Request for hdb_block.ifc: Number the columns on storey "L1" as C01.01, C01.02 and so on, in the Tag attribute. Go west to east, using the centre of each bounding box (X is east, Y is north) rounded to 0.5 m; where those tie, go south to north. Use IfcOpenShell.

First a look at what the model holds.

```python
import ifcopenshell
import ifcopenshell.util.element
import ifcopenshell.util.placement

model = ifcopenshell.open("hdb_block.ifc")
print(model.schema)
storey = next(s for s in model.by_type("IfcBuildingStorey") if s.Name == "L1")
columns = [e for e in ifcopenshell.util.element.get_decomposition(storey) if e.is_a("IfcColumn")]
for e in sorted(columns, key=lambda e: e.id()):
    origin = ifcopenshell.util.placement.get_local_placement(e.ObjectPlacement)[:3, 3]
    print(e.id(), e.Tag, e.Name, origin.round(2) + 0.0, sep=" | ")
```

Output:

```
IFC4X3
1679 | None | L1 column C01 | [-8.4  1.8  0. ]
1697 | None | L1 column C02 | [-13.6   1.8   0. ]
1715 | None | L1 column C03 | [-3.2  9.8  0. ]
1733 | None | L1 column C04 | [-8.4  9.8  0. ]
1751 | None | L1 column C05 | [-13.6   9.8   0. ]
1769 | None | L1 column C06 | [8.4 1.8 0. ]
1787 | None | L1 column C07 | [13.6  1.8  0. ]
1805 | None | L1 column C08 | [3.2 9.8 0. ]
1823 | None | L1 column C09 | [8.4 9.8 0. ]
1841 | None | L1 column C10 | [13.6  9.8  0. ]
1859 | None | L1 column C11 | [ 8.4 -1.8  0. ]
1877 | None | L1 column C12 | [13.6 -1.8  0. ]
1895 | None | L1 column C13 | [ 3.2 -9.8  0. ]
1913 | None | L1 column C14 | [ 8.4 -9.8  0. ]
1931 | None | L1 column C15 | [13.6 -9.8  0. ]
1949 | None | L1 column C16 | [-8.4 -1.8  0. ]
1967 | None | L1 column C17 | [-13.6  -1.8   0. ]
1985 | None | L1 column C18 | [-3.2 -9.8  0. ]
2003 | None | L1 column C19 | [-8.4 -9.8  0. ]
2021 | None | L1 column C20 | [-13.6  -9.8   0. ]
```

```python
import ifcopenshell
import ifcopenshell.geom
import ifcopenshell.util.element
import ifcopenshell.util.shape

model = ifcopenshell.open("hdb_block.ifc")
settings = ifcopenshell.geom.settings()
settings.set("use-world-coords", True)


def centre(element):
    shape = ifcopenshell.geom.create_shape(settings, element)
    return ifcopenshell.util.shape.get_bbox_centroid(shape.geometry)


storey = next(s for s in model.by_type("IfcBuildingStorey") if s.Name == "L1")
columns = [e for e in ifcopenshell.util.element.get_decomposition(storey) if e.is_a("IfcColumn")]

# Insertion points can sit at a corner or the storey origin, so sort by the geometry (in metres).
centres = {e: centre(e) for e in columns}
columns.sort(key=lambda e: (round(centres[e][0] / 0.5), centres[e][1]))

for i, e in enumerate(columns, start=1):
    number = f"C01.{i:02d}"
    e.Tag = number
    print(e.id(), number)

model.write("hdb_block-out.ifc")
```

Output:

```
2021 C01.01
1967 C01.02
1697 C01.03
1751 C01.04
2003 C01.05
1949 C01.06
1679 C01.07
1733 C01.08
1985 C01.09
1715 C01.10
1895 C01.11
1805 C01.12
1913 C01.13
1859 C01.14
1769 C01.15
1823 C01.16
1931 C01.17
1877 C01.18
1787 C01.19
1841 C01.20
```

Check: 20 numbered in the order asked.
